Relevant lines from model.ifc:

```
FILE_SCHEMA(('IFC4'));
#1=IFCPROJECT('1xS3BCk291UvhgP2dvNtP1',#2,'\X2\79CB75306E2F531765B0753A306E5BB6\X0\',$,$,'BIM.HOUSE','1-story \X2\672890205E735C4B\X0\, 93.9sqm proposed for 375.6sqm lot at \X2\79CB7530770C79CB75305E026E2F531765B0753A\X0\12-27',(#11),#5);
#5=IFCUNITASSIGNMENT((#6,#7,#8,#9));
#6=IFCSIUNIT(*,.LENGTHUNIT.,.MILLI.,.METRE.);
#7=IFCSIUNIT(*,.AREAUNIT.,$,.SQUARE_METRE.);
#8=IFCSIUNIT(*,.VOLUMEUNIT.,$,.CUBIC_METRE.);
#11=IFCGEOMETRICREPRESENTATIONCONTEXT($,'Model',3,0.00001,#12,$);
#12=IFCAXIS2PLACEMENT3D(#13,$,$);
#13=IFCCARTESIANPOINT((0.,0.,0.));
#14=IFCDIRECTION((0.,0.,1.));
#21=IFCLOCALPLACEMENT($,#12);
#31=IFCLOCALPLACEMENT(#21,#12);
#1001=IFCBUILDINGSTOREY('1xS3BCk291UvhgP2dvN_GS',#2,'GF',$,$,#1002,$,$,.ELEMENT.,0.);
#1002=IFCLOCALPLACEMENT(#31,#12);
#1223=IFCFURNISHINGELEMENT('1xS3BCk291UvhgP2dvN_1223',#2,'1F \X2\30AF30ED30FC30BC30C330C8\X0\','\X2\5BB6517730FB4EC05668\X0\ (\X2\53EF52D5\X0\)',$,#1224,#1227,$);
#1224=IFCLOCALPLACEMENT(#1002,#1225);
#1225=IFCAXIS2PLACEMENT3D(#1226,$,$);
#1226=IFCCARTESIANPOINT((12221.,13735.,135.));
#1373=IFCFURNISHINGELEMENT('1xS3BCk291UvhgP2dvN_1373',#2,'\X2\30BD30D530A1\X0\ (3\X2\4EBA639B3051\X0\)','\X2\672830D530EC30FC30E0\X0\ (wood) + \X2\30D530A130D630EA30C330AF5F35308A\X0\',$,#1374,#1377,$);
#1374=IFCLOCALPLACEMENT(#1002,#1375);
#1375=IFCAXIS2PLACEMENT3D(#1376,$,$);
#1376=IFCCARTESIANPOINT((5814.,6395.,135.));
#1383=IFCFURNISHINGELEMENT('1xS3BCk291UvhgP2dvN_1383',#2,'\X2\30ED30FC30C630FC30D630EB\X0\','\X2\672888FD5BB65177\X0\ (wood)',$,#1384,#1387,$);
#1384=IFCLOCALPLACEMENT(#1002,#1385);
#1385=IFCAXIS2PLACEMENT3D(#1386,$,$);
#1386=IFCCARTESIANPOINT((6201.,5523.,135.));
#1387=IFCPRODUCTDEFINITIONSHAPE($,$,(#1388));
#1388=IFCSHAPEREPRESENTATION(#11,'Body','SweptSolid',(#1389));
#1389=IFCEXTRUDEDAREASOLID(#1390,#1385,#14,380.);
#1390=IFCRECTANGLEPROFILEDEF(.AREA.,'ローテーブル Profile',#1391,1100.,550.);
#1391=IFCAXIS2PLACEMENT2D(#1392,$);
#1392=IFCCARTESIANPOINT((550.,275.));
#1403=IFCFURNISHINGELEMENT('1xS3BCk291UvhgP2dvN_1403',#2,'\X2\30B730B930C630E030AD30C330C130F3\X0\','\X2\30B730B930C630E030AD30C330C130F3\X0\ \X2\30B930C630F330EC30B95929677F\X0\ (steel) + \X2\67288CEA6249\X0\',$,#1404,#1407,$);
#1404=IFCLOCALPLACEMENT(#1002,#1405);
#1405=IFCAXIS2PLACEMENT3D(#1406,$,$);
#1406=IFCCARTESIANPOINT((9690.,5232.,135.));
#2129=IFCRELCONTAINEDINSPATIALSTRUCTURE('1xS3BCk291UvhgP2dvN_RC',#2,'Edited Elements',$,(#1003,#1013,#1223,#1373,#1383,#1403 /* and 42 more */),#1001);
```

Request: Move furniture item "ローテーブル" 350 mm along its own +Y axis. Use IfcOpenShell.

```python
import ifcopenshell
import ifcopenshell.api.geometry
import ifcopenshell.util.placement
import ifcopenshell.util.unit

model = ifcopenshell.open("model.ifc")
unit_scale = ifcopenshell.util.unit.calculate_unit_scale(model)

item = model.by_id(1383)
matrix = ifcopenshell.util.placement.get_local_placement(item.ObjectPlacement)
matrix[:3, 3] += matrix[:3, 1] * 0.35 / unit_scale
ifcopenshell.api.geometry.edit_object_placement(model, product=item, matrix=matrix, is_si=False)

print(ifcopenshell.util.placement.get_local_placement(item.ObjectPlacement).round(3) + 0.0)

model.write("model_v2.ifc")
```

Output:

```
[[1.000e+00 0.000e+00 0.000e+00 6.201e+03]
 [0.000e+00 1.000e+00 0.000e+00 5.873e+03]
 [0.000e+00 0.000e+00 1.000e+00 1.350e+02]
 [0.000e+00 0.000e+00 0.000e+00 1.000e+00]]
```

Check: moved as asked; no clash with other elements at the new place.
